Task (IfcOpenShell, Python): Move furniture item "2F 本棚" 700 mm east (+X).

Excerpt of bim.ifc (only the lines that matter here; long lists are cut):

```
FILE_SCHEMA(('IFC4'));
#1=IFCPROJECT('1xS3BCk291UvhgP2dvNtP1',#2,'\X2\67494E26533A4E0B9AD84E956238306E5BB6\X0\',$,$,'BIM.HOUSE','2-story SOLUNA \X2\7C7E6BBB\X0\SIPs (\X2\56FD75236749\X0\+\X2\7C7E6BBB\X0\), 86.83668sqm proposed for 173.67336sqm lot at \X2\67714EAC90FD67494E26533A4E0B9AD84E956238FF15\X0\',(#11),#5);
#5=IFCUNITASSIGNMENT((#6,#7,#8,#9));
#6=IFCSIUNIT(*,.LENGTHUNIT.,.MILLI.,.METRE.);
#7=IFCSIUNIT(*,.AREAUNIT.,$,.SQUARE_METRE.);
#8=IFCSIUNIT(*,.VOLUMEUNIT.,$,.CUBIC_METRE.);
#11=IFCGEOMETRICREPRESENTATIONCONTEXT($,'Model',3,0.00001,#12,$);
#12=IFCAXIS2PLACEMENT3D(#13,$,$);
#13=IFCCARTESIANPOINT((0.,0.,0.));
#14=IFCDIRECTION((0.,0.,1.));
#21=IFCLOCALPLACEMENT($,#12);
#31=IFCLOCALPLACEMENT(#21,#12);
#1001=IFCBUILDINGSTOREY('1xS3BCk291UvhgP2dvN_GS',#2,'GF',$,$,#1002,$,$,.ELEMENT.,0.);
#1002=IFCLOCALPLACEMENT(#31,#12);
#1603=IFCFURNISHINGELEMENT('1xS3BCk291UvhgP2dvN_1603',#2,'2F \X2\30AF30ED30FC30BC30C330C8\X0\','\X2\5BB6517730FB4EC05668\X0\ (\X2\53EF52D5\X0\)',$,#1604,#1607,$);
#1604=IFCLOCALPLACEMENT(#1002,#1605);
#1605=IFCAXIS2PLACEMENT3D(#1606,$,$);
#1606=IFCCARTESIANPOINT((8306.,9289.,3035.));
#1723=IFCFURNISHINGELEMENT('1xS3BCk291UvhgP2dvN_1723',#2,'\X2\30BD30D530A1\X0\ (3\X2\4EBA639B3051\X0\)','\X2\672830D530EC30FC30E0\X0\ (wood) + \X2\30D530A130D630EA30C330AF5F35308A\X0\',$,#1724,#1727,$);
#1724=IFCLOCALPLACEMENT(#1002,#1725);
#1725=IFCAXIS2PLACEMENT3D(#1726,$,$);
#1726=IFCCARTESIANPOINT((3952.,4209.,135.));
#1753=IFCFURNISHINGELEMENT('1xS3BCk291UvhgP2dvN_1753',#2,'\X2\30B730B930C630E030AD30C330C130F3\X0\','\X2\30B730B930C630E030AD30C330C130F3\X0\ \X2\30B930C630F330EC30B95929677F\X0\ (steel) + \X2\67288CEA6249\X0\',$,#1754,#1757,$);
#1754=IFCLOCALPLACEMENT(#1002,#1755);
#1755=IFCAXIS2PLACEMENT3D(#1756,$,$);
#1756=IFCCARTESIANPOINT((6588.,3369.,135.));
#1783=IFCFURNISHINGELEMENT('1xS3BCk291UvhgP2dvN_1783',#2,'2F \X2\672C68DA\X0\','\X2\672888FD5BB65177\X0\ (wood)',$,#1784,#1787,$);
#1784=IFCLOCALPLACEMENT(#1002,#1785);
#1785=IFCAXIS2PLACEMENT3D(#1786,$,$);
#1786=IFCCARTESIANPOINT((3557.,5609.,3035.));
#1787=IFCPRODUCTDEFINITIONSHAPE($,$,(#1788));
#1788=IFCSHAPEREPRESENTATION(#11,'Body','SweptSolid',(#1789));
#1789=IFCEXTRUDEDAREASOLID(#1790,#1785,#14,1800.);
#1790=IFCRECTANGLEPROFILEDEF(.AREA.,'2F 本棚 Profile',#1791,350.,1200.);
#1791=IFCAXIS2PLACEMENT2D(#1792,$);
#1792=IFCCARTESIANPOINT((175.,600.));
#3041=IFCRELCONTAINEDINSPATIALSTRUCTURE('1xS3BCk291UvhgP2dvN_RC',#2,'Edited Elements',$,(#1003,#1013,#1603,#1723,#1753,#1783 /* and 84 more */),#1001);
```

```python
import ifcopenshell
import ifcopenshell.api.geometry
import ifcopenshell.util.placement

model = ifcopenshell.open("bim.ifc")

item = model.by_guid("1xS3BCk291UvhgP2dvN_1783")
matrix = ifcopenshell.util.placement.get_local_placement(item.ObjectPlacement)
matrix[0, 3] += 700.0
ifcopenshell.api.geometry.edit_object_placement(model, product=item, matrix=matrix, is_si=False)

print(ifcopenshell.util.placement.get_local_placement(item.ObjectPlacement).round(3) + 0.0)

model.write("bim_edited.ifc")
```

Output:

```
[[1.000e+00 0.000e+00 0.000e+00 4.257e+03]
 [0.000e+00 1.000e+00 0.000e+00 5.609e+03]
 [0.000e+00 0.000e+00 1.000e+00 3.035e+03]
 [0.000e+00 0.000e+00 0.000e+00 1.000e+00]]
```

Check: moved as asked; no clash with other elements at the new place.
